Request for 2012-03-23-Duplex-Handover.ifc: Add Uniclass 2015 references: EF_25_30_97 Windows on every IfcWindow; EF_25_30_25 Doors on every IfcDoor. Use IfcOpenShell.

First a look at what the model holds.

```python
import ifcopenshell

model = ifcopenshell.open("2012-03-23-Duplex-Handover.ifc")
print(model.schema)
print("classifications:", [c.Name for c in model.by_type("IfcClassification")])
for ifc_class in ("IfcDoor", "IfcRoof", "IfcStair", "IfcWall", "IfcWindow"):
    print(ifc_class, len(model.by_type(ifc_class)))
```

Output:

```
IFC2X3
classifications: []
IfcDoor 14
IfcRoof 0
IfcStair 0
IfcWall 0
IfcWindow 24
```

```python
import ifcopenshell
import ifcopenshell.api.classification

model = ifcopenshell.open("2012-03-23-Duplex-Handover.ifc")

# IFC2X3 requires Source and Edition and has no link from the project to the system.
system = model.create_entity("IfcClassification", Source="NBS", Edition="2015", Name="Uniclass 2015")

codes = {
    "IfcWindow": ("EF_25_30_97", "Windows"),
    "IfcDoor": ("EF_25_30_25", "Doors"),
}
for ifc_class, (code, name) in codes.items():
    products = model.by_type(ifc_class)
    ifcopenshell.api.classification.add_reference(
        model, products=products, classification=system, identification=code, name=name
    )
    print(code, len(products))

model.write("2012-03-23-Duplex-Handover_rev.ifc")
```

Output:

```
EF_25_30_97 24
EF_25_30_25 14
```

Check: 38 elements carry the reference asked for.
